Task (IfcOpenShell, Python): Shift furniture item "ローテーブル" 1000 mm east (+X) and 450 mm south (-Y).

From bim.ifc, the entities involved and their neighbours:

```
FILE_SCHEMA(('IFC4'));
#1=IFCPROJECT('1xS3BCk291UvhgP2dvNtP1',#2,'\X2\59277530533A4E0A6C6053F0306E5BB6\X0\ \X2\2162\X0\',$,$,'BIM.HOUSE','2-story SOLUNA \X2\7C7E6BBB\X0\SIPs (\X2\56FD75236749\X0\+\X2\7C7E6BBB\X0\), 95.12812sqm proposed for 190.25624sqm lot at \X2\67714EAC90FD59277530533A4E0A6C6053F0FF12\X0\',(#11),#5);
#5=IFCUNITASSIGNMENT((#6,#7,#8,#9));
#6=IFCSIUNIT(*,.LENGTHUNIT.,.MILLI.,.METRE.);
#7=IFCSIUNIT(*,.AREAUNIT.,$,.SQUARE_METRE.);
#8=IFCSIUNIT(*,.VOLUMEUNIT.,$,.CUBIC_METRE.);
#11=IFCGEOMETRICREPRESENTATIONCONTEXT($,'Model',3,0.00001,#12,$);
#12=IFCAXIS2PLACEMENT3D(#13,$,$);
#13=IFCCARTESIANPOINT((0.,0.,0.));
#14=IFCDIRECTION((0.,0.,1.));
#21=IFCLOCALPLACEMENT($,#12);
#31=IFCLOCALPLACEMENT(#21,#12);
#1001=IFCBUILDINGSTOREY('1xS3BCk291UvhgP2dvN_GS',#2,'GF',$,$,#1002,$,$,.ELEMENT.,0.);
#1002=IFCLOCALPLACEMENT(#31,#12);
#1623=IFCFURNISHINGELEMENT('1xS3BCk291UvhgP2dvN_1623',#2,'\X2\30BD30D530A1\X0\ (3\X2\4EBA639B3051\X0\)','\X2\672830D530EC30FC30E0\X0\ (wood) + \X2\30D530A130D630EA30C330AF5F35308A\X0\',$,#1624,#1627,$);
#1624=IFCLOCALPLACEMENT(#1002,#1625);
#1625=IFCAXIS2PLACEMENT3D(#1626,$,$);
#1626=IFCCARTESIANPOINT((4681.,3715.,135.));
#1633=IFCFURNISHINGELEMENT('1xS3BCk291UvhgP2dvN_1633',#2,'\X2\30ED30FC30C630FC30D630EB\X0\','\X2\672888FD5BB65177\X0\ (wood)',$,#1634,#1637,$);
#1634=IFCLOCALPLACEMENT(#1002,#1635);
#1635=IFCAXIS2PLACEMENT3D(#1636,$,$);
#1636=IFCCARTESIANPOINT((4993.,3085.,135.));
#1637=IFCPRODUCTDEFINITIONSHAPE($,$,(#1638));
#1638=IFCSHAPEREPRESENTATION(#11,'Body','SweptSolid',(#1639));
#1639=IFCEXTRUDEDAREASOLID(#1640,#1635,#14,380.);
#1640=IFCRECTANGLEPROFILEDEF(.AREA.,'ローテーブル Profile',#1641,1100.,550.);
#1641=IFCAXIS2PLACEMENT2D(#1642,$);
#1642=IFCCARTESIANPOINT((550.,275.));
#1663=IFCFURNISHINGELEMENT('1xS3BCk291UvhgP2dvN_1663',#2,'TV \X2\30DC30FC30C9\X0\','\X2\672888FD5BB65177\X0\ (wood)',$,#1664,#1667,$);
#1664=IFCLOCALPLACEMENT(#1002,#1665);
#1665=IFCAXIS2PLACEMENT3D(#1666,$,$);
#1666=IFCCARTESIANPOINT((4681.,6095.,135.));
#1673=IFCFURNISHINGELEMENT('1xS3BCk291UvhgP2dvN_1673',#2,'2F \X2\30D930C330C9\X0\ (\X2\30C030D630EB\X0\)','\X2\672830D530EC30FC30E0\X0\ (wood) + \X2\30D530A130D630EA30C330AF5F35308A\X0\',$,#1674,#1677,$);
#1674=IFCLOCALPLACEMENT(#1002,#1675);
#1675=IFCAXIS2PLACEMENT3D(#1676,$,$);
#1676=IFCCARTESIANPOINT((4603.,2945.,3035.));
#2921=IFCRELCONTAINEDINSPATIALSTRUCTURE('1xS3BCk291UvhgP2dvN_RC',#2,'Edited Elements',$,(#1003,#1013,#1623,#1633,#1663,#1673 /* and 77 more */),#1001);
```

```python
import ifcopenshell
import ifcopenshell.api.geometry
import ifcopenshell.util.placement
import ifcopenshell.util.unit

model = ifcopenshell.open("bim.ifc")
unit_scale = ifcopenshell.util.unit.calculate_unit_scale(model)

item = model.by_id(1633)
matrix = ifcopenshell.util.placement.get_local_placement(item.ObjectPlacement)
matrix[0, 3] += 1 / unit_scale
matrix[1, 3] -= 0.45 / unit_scale
ifcopenshell.api.geometry.edit_object_placement(model, product=item, matrix=matrix, is_si=False)

print(ifcopenshell.util.placement.get_local_placement(item.ObjectPlacement).round(3) + 0.0)

model.write("bim_rev.ifc")
```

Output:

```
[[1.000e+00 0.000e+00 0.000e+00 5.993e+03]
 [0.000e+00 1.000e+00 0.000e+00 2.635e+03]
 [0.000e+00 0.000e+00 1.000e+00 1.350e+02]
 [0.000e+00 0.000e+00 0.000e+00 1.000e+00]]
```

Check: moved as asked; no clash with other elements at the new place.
